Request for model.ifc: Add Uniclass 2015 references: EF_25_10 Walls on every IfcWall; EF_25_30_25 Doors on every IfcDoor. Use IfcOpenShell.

First a look at what the model holds.

```python
import ifcopenshell

model = ifcopenshell.open("model.ifc")
print(model.schema)
print("classifications:", [c.Name for c in model.by_type("IfcClassification")])
for ifc_class in ("IfcDoor", "IfcRoof", "IfcStair", "IfcWall", "IfcWindow"):
    print(ifc_class, len(model.by_type(ifc_class)))
```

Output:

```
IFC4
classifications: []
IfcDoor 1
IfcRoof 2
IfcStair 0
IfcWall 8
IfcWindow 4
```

```python
import ifcopenshell
import ifcopenshell.api.classification

model = ifcopenshell.open("model.ifc")

system = ifcopenshell.api.classification.add_classification(model, classification="Uniclass 2015")

codes = {
    "IfcWall": ("EF_25_10", "Walls"),
    "IfcDoor": ("EF_25_30_25", "Doors"),
}
for ifc_class, (code, name) in codes.items():
    products = model.by_type(ifc_class)
    ifcopenshell.api.classification.add_reference(
        model, products=products, classification=system, identification=code, name=name
    )
    print(code, len(products))

model.write("model-out.ifc")
```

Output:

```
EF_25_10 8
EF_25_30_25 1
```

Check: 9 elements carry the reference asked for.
